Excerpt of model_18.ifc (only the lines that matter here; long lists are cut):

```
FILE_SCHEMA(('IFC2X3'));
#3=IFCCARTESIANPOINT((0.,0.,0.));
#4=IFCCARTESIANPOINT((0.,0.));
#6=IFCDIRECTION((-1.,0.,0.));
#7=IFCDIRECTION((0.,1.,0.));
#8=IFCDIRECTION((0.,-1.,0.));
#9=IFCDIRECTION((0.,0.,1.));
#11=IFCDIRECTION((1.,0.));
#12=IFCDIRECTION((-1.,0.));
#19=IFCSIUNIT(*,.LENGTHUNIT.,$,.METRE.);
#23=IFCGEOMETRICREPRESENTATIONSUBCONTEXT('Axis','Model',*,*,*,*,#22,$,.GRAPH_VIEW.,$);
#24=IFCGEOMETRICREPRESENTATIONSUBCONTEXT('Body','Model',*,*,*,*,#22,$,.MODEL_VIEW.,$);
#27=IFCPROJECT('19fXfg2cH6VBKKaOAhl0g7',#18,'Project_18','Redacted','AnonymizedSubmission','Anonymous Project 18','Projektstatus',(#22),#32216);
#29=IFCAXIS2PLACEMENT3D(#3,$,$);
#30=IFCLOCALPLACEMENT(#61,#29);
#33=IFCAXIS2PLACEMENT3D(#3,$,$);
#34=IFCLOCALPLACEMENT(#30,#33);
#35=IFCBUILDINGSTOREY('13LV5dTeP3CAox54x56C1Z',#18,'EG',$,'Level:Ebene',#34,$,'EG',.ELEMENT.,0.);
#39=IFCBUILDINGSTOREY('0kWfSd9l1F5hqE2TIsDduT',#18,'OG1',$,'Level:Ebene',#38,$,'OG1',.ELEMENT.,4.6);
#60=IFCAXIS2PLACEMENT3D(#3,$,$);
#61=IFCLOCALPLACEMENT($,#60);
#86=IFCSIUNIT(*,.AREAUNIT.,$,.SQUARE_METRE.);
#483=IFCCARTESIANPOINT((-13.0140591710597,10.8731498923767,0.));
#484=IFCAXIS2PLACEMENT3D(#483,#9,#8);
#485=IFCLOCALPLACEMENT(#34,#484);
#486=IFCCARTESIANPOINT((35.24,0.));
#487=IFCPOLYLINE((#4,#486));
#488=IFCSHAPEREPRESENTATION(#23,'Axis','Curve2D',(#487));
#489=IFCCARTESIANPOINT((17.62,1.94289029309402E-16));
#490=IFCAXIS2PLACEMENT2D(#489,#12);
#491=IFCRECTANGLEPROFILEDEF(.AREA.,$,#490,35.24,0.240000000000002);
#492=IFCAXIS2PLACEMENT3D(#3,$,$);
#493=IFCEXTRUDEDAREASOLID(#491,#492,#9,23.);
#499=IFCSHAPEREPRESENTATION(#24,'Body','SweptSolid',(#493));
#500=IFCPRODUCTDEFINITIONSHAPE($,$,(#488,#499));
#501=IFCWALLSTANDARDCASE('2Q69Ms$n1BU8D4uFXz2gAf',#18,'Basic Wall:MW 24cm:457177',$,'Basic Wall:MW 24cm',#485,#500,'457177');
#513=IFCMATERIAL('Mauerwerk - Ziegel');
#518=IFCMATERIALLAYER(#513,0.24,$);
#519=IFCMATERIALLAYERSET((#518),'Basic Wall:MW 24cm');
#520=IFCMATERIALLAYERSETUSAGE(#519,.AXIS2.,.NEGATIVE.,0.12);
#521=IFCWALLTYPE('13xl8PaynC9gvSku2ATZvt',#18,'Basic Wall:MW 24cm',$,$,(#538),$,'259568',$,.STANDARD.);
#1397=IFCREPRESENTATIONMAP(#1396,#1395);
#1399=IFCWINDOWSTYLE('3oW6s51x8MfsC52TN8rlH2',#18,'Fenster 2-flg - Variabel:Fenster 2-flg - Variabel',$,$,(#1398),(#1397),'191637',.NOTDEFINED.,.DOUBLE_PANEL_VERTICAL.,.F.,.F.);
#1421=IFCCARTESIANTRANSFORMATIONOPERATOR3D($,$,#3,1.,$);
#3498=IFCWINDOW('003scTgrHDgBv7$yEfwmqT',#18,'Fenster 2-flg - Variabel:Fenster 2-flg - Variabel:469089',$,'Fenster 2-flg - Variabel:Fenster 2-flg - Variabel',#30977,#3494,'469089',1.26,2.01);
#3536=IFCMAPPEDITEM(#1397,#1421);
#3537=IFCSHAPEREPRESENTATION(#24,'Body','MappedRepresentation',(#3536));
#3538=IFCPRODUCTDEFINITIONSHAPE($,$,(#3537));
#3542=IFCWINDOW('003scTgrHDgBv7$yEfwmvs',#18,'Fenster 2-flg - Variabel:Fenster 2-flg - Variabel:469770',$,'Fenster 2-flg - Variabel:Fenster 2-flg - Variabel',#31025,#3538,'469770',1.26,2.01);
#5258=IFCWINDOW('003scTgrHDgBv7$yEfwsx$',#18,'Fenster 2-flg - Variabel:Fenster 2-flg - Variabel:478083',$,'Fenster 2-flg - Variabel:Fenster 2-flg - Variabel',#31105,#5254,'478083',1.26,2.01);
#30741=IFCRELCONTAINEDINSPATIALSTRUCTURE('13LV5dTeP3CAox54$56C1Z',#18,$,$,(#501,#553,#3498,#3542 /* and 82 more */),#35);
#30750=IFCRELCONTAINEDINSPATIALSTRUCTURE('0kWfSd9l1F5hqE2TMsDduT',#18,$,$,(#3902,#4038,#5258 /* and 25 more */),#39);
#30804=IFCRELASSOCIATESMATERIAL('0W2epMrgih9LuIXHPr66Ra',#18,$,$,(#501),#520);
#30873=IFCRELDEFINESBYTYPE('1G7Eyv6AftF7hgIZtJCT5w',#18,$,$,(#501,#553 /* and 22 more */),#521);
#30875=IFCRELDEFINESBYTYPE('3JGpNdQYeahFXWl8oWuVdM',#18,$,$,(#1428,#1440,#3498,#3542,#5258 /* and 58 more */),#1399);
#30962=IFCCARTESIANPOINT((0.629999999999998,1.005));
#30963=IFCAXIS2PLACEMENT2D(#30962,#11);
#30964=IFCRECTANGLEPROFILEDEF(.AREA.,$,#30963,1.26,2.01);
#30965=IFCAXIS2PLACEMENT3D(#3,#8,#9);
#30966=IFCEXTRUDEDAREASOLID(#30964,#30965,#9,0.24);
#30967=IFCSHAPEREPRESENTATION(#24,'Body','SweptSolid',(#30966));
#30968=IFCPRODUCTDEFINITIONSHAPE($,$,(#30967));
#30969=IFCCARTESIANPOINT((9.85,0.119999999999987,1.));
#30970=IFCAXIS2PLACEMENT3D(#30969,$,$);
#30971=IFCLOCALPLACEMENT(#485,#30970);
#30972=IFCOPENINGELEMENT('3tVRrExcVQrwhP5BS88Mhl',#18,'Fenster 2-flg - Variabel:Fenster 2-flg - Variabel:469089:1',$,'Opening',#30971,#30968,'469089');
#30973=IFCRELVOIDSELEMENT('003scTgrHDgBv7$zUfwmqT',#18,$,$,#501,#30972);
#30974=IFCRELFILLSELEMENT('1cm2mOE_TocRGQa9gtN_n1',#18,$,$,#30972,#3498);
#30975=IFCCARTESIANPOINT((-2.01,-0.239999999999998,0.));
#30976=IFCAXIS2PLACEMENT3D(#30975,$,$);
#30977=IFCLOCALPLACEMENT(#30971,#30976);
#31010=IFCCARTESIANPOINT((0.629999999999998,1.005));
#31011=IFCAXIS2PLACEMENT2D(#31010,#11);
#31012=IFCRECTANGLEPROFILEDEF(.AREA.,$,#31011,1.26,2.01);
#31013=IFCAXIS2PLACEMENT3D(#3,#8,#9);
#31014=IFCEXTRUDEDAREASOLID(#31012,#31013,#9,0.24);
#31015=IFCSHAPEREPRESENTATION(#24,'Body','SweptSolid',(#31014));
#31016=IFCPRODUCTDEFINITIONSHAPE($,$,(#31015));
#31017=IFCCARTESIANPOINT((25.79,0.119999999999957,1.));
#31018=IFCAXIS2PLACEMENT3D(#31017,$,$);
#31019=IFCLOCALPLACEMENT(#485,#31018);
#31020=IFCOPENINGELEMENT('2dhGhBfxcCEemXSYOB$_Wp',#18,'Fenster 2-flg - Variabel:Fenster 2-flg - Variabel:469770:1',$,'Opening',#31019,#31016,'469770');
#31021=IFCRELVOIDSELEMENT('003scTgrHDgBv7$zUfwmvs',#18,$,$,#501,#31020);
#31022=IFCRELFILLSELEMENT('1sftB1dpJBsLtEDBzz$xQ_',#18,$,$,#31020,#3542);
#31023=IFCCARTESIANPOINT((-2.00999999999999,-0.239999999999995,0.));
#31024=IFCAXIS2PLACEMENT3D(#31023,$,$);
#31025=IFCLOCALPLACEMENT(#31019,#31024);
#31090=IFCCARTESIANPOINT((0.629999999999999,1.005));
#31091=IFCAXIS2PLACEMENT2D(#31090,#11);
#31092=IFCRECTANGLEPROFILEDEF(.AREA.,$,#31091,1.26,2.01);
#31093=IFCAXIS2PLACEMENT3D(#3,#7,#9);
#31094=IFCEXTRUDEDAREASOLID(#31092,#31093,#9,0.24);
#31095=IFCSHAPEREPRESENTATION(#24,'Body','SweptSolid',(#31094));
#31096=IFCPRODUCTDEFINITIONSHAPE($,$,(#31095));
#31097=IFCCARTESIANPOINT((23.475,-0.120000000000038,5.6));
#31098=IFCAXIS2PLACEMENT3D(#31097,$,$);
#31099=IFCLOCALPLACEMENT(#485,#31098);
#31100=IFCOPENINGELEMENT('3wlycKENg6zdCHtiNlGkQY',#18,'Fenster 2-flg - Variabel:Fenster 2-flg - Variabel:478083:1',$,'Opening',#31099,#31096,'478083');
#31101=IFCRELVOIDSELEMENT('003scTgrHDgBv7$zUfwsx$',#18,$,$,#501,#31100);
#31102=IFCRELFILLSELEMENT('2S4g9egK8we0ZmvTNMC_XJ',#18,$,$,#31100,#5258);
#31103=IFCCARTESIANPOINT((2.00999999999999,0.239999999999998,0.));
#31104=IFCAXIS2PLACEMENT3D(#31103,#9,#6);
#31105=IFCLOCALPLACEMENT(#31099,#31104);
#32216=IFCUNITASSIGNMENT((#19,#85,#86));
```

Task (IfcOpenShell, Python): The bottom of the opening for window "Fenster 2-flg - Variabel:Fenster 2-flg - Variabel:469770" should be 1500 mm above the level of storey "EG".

```python
import numpy as np
import ifcopenshell
import ifcopenshell.api.geometry
import ifcopenshell.geom
import ifcopenshell.util.element
import ifcopenshell.util.placement
import ifcopenshell.util.shape
import ifcopenshell.util.unit

model = ifcopenshell.open("model_18.ifc")
unit_scale = ifcopenshell.util.unit.calculate_unit_scale(model)

window = model.by_id(3542)
opening = window.FillsVoids[0].RelatingOpeningElement
storey = ifcopenshell.util.element.get_container(window, ifc_class="IfcBuildingStorey")
level = ifcopenshell.util.placement.get_local_placement(storey.ObjectPlacement)[2, 3]

# The opening's origin need not be at the sill, so measure its lowest point.
shape = ifcopenshell.geom.create_shape(ifcopenshell.geom.settings(), opening)
bottom = ifcopenshell.util.shape.get_shape_bottom_elevation(shape, shape.geometry) / unit_scale
dz = level + 1.5 - bottom

shift = np.array([0.0, 0.0, dz])
# The window is placed relative to its opening, so it follows when the opening moves.
matrix = ifcopenshell.util.placement.get_local_placement(opening.ObjectPlacement)
matrix[:3, 3] += shift
ifcopenshell.api.geometry.edit_object_placement(
    model, product=opening, matrix=matrix, is_si=False, should_transform_children=True
)

print(f"moved by {dz * unit_scale:+.3f} m")

model.write("model_18-out.ifc")
```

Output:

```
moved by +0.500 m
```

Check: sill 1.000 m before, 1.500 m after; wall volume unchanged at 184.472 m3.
